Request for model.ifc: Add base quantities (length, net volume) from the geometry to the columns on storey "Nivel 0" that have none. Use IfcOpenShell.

First a look at what the model holds.

```python
import ifcopenshell
import ifcopenshell.util.element
import ifcopenshell.util.unit

model = ifcopenshell.open("model.ifc")
print(model.schema)
for unit_type in ("LENGTHUNIT", "AREAUNIT", "VOLUMEUNIT"):
    print(unit_type, ifcopenshell.util.unit.calculate_unit_scale(model, unit_type))
storey = next(s for s in model.by_type("IfcBuildingStorey") if s.Name == "Nivel 0")
columns = [e for e in ifcopenshell.util.element.get_decomposition(storey) if e.is_a("IfcColumn")]
for e in sorted(columns, key=lambda e: e.id()):
    print(e.id(), e.is_a(), e.Name, list(ifcopenshell.util.element.get_psets(e, qtos_only=True)), sep=" | ")
```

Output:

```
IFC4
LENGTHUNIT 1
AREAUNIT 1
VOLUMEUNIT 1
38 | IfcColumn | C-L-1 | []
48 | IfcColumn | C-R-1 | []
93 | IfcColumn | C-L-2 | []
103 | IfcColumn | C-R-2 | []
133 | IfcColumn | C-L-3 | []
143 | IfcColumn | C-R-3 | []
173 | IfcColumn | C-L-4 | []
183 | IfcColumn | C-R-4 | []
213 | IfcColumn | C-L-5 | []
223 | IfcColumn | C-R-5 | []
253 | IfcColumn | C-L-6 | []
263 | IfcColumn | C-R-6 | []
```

```python
import ifcopenshell
import ifcopenshell.api.pset
import ifcopenshell.geom
import ifcopenshell.util.element
import ifcopenshell.util.shape
import ifcopenshell.util.unit

model = ifcopenshell.open("model.ifc")
unit_scale = ifcopenshell.util.unit.calculate_unit_scale(model)
volume_scale = ifcopenshell.util.unit.calculate_unit_scale(model, "VOLUMEUNIT")
settings = ifcopenshell.geom.settings()

storey = next(s for s in model.by_type("IfcBuildingStorey") if s.Name == "Nivel 0")
columns = [e for e in ifcopenshell.util.element.get_decomposition(storey) if e.is_a("IfcColumn")]

for e in sorted(columns, key=lambda e: e.id()):
    if ifcopenshell.util.element.get_psets(e, qtos_only=True, should_inherit=False):
        continue
    # Geometry comes back in metres, in the element's own axes.
    shape = ifcopenshell.geom.create_shape(settings, e)
    values = {
        "Length": ifcopenshell.util.shape.get_z(shape.geometry) / unit_scale,
        "NetVolume": ifcopenshell.util.shape.get_volume(shape.geometry) / volume_scale,
    }
    qto = ifcopenshell.api.pset.add_qto(model, product=e, name="Qto_ColumnBaseQuantities")
    ifcopenshell.api.pset.edit_qto(model, qto=qto, properties=values)
    print(e.id(), {k: round(v, 3) for k, v in values.items()})

model.write("model-out.ifc")
```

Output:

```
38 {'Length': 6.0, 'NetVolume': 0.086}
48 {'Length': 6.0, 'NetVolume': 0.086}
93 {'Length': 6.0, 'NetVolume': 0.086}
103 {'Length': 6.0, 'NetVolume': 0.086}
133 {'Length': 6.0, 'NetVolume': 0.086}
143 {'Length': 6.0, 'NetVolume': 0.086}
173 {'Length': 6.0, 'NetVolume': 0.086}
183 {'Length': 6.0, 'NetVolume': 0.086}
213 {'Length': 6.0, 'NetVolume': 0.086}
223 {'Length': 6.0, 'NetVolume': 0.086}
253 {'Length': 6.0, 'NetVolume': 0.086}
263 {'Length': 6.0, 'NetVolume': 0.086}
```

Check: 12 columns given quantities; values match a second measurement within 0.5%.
